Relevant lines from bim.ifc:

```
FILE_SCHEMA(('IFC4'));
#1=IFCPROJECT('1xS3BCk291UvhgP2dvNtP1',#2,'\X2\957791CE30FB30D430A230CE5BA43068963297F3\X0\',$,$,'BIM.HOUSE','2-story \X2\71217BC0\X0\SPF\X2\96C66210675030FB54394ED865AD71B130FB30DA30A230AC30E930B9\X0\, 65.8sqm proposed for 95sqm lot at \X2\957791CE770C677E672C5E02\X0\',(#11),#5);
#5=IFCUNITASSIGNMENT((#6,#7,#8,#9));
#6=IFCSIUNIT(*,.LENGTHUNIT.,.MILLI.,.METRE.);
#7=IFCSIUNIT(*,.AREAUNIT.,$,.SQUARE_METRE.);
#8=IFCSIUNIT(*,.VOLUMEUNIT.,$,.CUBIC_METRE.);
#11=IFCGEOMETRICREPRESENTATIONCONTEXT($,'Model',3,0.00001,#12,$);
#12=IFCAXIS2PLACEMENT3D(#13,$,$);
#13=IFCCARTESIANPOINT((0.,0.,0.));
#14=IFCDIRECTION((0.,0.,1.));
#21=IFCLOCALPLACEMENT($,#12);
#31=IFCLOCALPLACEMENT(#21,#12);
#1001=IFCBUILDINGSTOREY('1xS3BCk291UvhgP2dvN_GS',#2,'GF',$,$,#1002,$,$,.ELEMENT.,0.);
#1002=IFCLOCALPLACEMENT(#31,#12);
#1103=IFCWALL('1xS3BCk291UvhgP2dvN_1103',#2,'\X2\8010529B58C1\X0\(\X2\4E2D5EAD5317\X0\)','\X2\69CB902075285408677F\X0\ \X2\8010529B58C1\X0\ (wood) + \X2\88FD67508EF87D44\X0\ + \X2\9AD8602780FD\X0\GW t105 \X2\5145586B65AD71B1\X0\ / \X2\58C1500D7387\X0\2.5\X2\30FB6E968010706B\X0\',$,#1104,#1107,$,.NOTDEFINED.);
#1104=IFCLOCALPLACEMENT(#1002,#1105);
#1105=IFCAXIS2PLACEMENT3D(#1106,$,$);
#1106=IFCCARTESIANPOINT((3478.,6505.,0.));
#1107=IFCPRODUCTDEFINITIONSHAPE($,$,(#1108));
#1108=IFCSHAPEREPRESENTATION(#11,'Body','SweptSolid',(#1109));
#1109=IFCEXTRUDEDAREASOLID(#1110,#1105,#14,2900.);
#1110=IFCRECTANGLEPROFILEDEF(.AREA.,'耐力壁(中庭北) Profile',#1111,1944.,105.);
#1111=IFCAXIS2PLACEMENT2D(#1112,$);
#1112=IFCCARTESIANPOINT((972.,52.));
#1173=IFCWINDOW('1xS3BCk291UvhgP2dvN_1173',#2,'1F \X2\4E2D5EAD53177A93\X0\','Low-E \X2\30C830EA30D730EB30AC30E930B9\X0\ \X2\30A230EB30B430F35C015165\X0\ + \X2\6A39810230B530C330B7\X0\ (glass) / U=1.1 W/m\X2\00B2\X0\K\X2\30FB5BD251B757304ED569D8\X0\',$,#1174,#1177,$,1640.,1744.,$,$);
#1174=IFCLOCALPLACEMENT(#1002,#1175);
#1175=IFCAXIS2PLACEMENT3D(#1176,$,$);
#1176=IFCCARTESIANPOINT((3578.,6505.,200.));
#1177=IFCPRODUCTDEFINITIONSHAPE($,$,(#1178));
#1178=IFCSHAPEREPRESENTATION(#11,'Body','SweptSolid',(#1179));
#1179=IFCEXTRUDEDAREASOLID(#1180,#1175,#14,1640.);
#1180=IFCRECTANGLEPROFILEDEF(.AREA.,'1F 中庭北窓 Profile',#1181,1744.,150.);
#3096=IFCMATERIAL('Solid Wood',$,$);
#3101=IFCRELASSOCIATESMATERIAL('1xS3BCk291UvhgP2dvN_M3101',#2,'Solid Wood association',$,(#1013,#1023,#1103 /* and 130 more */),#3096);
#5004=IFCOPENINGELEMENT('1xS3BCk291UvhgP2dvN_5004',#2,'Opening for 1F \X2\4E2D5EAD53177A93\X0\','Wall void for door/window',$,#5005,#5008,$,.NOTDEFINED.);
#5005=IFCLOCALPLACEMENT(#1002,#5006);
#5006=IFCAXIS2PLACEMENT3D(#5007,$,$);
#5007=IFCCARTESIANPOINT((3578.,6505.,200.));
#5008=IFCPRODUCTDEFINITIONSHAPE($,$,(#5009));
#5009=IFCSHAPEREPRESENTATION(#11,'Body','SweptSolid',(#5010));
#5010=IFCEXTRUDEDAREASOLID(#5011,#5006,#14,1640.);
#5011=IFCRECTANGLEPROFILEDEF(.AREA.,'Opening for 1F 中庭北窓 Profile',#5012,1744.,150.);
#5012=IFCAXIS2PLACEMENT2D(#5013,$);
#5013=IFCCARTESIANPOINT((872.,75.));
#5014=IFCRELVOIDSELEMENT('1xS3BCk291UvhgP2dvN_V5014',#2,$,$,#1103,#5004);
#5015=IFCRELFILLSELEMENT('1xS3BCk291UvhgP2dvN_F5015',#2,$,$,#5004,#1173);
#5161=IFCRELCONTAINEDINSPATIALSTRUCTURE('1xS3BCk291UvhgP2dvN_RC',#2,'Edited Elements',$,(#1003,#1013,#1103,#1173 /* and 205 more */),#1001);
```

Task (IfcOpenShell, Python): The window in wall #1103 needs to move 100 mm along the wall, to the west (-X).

```python
import ifcopenshell
import ifcopenshell.api.geometry
import ifcopenshell.util.placement
import ifcopenshell.util.unit

model = ifcopenshell.open("bim.ifc")
unit_scale = ifcopenshell.util.unit.calculate_unit_scale(model)

window = model.by_guid("1xS3BCk291UvhgP2dvN_1173")
opening = window.FillsVoids[0].RelatingOpeningElement
wall = opening.VoidsElements[0].RelatingBuildingElement

wall_matrix = ifcopenshell.util.placement.get_local_placement(wall.ObjectPlacement)
shift = wall_matrix[:3, 0] * -0.1 / unit_scale
before = ifcopenshell.util.placement.get_local_placement(window.ObjectPlacement)[:3, 3].copy()

# The window is not placed relative to its opening, so move both.
for product in (opening, window):
    matrix = ifcopenshell.util.placement.get_local_placement(product.ObjectPlacement)
    matrix[:3, 3] += shift
    ifcopenshell.api.geometry.edit_object_placement(model, product=product, matrix=matrix, is_si=False)

after = ifcopenshell.util.placement.get_local_placement(window.ObjectPlacement)[:3, 3]
print("window moved by", (after - before).round(3) + 0.0)

model.write("bim_updated.ifc")
```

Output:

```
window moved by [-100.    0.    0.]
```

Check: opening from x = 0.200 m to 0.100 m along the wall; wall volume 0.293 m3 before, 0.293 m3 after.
